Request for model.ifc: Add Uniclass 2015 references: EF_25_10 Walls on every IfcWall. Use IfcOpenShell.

First a look at what the model holds.

```python
import ifcopenshell

model = ifcopenshell.open("model.ifc")
print(model.schema)
print("classifications:", [c.Name for c in model.by_type("IfcClassification")])
for ifc_class in ("IfcDoor", "IfcRoof", "IfcStair", "IfcWall", "IfcWindow"):
    print(ifc_class, len(model.by_type(ifc_class)))
```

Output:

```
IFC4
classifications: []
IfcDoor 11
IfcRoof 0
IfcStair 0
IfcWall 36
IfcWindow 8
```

```python
import ifcopenshell
import ifcopenshell.api.classification

model = ifcopenshell.open("model.ifc")

system = ifcopenshell.api.classification.add_classification(model, classification="Uniclass 2015")

codes = {
    "IfcWall": ("EF_25_10", "Walls"),
}
for ifc_class, (code, name) in codes.items():
    products = model.by_type(ifc_class)
    ifcopenshell.api.classification.add_reference(
        model, products=products, classification=system, identification=code, name=name
    )
    print(code, len(products))

model.write("model_updated.ifc")
```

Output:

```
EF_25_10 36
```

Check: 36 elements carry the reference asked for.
